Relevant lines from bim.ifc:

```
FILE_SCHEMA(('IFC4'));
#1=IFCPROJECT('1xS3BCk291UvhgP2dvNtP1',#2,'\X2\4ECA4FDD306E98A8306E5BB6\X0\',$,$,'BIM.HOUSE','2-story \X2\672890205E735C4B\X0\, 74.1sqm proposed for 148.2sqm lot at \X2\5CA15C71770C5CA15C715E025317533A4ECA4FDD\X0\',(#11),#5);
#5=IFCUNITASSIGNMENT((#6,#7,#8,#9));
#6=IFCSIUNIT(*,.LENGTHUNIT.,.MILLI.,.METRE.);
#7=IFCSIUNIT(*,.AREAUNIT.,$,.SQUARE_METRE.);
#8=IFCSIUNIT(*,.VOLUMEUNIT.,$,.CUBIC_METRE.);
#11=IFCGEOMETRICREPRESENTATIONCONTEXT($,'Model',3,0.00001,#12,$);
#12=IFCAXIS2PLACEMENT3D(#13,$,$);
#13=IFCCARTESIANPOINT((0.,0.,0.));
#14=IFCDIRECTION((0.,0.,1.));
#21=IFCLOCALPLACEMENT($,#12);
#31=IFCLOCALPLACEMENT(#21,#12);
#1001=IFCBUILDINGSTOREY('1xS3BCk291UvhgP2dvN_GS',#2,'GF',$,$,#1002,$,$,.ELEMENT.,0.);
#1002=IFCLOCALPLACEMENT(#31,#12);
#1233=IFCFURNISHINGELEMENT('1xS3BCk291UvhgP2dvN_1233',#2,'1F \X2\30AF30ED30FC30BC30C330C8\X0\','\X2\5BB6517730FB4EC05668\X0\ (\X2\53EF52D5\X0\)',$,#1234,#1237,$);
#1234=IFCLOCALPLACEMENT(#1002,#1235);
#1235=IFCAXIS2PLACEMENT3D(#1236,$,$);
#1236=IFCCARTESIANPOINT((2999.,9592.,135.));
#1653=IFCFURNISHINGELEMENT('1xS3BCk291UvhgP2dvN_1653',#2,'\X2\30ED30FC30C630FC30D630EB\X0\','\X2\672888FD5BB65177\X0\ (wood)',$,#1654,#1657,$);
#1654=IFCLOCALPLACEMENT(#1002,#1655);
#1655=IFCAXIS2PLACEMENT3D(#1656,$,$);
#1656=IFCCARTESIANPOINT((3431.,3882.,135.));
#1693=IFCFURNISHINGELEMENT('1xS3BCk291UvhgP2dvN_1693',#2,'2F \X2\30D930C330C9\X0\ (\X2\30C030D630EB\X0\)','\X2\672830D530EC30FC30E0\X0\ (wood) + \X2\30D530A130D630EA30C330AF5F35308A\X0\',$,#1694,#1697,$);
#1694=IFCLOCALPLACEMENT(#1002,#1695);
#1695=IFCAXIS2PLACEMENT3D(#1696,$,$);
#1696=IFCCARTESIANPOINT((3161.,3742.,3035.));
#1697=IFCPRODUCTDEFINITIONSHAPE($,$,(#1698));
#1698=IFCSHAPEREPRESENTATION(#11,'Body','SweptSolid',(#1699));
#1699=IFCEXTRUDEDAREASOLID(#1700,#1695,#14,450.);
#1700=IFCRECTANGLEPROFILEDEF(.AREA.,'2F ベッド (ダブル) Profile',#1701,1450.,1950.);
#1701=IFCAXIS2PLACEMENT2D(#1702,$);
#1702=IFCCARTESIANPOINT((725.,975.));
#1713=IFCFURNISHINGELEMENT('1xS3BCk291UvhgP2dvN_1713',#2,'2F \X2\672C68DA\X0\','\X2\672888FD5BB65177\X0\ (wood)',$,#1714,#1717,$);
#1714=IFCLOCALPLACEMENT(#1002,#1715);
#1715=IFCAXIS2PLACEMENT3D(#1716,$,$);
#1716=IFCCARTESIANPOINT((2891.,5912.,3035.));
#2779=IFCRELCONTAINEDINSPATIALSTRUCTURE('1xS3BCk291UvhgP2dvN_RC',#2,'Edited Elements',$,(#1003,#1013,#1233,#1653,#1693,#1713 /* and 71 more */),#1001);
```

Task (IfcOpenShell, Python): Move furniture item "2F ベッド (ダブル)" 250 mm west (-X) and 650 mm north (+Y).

```python
import ifcopenshell
import ifcopenshell.api.geometry
import ifcopenshell.util.placement
import ifcopenshell.util.unit

model = ifcopenshell.open("bim.ifc")
unit_scale = ifcopenshell.util.unit.calculate_unit_scale(model)

item = model.by_guid("1xS3BCk291UvhgP2dvN_1693")
matrix = ifcopenshell.util.placement.get_local_placement(item.ObjectPlacement)
matrix[0, 3] -= 0.25 / unit_scale
matrix[1, 3] += 0.65 / unit_scale
ifcopenshell.api.geometry.edit_object_placement(model, product=item, matrix=matrix, is_si=False)

print(ifcopenshell.util.placement.get_local_placement(item.ObjectPlacement).round(3) + 0.0)

model.write("bim_v2.ifc")
```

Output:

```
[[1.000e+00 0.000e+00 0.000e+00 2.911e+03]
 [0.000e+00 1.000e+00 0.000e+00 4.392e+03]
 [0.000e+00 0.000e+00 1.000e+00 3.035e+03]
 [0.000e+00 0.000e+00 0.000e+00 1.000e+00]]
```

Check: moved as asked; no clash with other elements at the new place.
